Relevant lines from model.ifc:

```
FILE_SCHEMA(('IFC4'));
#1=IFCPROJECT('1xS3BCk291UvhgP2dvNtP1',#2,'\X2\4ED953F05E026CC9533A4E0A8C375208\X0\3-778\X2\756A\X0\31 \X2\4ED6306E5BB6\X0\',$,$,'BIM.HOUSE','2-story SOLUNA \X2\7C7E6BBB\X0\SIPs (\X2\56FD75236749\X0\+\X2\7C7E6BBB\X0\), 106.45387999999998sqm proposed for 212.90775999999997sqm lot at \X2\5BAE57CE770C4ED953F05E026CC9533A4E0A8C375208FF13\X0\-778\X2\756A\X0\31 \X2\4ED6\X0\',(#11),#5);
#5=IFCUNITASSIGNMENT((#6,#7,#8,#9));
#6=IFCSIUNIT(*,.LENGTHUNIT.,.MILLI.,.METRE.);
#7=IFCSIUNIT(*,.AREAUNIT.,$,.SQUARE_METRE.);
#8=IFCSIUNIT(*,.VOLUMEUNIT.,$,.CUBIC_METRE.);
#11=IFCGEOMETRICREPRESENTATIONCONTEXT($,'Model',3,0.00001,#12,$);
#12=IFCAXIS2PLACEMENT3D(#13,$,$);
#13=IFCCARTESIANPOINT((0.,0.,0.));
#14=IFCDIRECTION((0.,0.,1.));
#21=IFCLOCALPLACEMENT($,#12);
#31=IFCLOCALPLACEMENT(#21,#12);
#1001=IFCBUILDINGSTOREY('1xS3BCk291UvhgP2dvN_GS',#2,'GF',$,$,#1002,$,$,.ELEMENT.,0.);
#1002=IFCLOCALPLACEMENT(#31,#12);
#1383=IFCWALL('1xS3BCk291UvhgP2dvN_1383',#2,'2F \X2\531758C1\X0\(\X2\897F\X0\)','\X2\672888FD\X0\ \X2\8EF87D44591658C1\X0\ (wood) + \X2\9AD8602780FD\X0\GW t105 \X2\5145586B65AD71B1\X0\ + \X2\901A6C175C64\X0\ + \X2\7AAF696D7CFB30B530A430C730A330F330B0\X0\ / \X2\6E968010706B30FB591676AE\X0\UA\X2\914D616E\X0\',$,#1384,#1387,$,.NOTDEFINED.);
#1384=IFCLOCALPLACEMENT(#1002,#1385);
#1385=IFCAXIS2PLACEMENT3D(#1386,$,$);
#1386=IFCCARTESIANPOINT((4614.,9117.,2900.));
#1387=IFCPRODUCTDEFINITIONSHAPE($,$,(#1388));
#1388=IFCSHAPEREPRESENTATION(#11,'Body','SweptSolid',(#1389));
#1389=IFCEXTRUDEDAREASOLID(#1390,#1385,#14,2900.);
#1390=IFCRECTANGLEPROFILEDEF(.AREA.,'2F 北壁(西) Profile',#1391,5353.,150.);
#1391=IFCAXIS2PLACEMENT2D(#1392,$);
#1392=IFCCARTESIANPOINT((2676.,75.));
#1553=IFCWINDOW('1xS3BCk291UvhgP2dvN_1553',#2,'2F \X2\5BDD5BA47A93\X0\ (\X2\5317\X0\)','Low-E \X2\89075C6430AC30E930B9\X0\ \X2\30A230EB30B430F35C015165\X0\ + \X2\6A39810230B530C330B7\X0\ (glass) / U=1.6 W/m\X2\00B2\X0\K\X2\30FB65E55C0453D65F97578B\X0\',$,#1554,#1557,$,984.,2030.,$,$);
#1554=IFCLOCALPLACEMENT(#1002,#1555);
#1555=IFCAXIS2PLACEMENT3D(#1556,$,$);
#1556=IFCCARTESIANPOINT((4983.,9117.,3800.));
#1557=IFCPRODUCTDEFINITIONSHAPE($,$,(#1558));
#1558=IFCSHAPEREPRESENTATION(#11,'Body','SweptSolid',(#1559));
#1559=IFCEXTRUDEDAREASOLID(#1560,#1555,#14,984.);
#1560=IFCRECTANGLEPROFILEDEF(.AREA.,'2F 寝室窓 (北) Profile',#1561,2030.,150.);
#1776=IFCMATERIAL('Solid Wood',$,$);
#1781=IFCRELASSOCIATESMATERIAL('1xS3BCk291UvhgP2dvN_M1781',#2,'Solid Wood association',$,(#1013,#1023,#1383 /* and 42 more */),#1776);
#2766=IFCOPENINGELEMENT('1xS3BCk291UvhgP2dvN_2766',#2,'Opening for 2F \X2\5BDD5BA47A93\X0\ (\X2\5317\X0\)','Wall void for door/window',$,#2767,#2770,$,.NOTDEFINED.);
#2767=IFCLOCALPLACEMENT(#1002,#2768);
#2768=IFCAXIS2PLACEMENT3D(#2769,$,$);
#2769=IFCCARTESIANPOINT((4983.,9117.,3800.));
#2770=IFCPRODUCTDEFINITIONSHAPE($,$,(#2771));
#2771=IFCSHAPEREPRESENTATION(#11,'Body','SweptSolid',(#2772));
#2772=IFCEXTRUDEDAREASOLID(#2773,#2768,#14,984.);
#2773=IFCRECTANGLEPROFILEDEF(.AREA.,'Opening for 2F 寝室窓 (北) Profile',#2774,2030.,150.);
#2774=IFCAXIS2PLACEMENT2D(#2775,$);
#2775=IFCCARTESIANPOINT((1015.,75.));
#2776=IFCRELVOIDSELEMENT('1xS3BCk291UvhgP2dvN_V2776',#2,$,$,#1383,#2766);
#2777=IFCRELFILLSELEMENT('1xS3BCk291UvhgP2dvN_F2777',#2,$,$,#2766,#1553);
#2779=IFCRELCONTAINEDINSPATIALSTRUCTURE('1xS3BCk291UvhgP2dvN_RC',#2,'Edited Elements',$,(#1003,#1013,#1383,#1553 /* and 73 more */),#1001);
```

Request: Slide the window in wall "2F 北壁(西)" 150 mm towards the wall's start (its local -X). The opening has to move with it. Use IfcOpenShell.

```python
import ifcopenshell
import ifcopenshell.api.geometry
import ifcopenshell.util.placement
import ifcopenshell.util.unit

model = ifcopenshell.open("model.ifc")
unit_scale = ifcopenshell.util.unit.calculate_unit_scale(model)

window = model.by_guid("1xS3BCk291UvhgP2dvN_1553")
opening = window.FillsVoids[0].RelatingOpeningElement
wall = opening.VoidsElements[0].RelatingBuildingElement

wall_matrix = ifcopenshell.util.placement.get_local_placement(wall.ObjectPlacement)
shift = wall_matrix[:3, 0] * -0.15 / unit_scale
before = ifcopenshell.util.placement.get_local_placement(window.ObjectPlacement)[:3, 3].copy()

# The window is not placed relative to its opening, so move both.
for product in (opening, window):
    matrix = ifcopenshell.util.placement.get_local_placement(product.ObjectPlacement)
    matrix[:3, 3] += shift
    ifcopenshell.api.geometry.edit_object_placement(model, product=product, matrix=matrix, is_si=False)

after = ifcopenshell.util.placement.get_local_placement(window.ObjectPlacement)[:3, 3]
print("window moved by", (after - before).round(3) + 0.0)

model.write("model_rev.ifc")
```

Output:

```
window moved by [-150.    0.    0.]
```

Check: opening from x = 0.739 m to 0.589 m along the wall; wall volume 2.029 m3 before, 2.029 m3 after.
